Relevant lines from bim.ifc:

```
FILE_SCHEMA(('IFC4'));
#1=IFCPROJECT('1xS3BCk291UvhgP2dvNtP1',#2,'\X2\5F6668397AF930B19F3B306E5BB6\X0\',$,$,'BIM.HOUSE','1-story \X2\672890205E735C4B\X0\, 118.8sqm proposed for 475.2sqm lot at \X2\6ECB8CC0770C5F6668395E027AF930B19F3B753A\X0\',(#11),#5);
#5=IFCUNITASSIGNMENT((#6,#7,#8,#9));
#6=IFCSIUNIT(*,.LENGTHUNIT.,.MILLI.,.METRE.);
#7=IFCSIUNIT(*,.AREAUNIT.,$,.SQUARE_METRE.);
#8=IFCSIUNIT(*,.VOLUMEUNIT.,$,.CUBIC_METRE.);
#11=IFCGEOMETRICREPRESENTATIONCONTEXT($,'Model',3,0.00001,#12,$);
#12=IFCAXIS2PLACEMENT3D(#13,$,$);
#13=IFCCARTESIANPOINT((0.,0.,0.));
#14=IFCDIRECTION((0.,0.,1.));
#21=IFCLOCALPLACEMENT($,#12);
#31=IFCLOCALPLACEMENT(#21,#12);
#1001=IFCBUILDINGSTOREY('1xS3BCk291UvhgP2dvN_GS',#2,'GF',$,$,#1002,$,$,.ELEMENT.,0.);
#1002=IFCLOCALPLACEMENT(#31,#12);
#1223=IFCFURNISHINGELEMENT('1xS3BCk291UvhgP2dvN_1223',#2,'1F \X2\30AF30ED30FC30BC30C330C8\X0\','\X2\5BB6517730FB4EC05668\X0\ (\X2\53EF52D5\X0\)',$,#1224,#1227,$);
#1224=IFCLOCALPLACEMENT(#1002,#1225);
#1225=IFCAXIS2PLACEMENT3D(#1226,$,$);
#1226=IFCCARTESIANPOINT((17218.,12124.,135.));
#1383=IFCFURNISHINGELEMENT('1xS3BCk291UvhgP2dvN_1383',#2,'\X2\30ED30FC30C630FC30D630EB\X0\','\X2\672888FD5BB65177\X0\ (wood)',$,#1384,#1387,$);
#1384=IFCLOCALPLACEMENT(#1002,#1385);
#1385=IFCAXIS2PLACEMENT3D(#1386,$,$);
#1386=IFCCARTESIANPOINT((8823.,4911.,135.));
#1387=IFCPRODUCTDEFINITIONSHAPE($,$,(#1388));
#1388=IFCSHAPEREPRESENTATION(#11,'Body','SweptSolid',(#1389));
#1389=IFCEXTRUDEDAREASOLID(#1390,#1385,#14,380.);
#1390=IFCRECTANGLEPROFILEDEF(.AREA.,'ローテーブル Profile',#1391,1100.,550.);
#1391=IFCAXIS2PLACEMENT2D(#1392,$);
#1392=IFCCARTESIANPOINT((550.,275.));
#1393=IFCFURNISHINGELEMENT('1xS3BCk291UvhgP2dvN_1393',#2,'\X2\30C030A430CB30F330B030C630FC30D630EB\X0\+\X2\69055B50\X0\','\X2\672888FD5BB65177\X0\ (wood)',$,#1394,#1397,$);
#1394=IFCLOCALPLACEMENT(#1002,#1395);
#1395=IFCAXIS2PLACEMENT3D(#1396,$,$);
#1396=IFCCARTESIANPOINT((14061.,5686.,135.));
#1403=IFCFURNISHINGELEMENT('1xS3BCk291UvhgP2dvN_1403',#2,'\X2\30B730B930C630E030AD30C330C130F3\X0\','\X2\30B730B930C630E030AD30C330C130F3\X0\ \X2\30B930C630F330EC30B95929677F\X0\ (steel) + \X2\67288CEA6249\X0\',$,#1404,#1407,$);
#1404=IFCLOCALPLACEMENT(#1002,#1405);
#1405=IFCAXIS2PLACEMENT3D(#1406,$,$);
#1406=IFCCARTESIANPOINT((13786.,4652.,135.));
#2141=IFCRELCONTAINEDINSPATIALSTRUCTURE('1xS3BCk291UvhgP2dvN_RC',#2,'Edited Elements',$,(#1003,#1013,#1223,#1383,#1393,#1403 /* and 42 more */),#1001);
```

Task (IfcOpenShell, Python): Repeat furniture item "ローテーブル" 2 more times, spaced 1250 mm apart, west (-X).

```python
import numpy as np
import ifcopenshell
import ifcopenshell.api.geometry
import ifcopenshell.api.root
import ifcopenshell.util.element
import ifcopenshell.util.placement
import ifcopenshell.util.unit

model = ifcopenshell.open("bim.ifc")
unit_scale = ifcopenshell.util.unit.calculate_unit_scale(model)


def reuse_history(source, copy):
    """copy_class also copies each property set's owner history, people and application; keep the originals."""
    for rel in copy.IsDefinedBy:
        if rel.is_a("IfcRelDefinesByProperties") and (history := rel.RelatingPropertyDefinition.OwnerHistory):
            rel.RelatingPropertyDefinition.OwnerHistory = source.OwnerHistory
            ifcopenshell.util.element.remove_deep2(model, history)


source = model.by_id(1383)
base = ifcopenshell.util.placement.get_local_placement(source.ObjectPlacement)
step = np.array([-1.0, 0.0, 0.0]) * 1.25 / unit_scale

for i in range(1, 3):
    copy = ifcopenshell.api.root.copy_class(model, product=source)
    copy.Representation = ifcopenshell.util.element.copy_deep(
        model, source.Representation, exclude=["IfcGeometricRepresentationContext", "IfcRepresentationMap"]
    )
    reuse_history(source, copy)
    matrix = base.copy()
    matrix[:3, 3] += i * step
    print("added at", matrix[:3, 3].round(3) + 0.0)
    ifcopenshell.api.geometry.edit_object_placement(model, product=copy, matrix=matrix, is_si=False)

model.write("bim_edited.ifc")
```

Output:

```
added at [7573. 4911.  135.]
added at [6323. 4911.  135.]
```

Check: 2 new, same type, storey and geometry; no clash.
